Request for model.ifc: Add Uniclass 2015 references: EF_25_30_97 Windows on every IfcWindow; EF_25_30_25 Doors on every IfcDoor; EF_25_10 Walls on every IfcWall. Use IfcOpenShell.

First a look at what the model holds.

```python
import ifcopenshell

model = ifcopenshell.open("model.ifc")
print(model.schema)
print("classifications:", [c.Name for c in model.by_type("IfcClassification")])
for ifc_class in ("IfcDoor", "IfcRoof", "IfcStair", "IfcWall", "IfcWindow"):
    print(ifc_class, len(model.by_type(ifc_class)))
```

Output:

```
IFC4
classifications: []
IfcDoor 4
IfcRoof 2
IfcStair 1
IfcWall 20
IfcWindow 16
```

```python
import ifcopenshell
import ifcopenshell.api.classification

model = ifcopenshell.open("model.ifc")

system = ifcopenshell.api.classification.add_classification(model, classification="Uniclass 2015")

codes = {
    "IfcWindow": ("EF_25_30_97", "Windows"),
    "IfcDoor": ("EF_25_30_25", "Doors"),
    "IfcWall": ("EF_25_10", "Walls"),
}
for ifc_class, (code, name) in codes.items():
    products = model.by_type(ifc_class)
    ifcopenshell.api.classification.add_reference(
        model, products=products, classification=system, identification=code, name=name
    )
    print(code, len(products))

model.write("model_rev.ifc")
```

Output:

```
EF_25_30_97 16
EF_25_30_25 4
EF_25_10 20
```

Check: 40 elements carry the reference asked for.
